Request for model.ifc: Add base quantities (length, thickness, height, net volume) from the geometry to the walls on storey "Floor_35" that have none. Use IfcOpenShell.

First a look at what the model holds.

```python
import ifcopenshell
import ifcopenshell.util.element
import ifcopenshell.util.unit

model = ifcopenshell.open("model.ifc")
print(model.schema)
for unit_type in ("LENGTHUNIT", "AREAUNIT", "VOLUMEUNIT"):
    print(unit_type, ifcopenshell.util.unit.calculate_unit_scale(model, unit_type))
storey = next(s for s in model.by_type("IfcBuildingStorey") if s.Name == "Floor_35")
walls = [e for e in ifcopenshell.util.element.get_decomposition(storey) if e.is_a("IfcWall")]
for e in sorted(walls, key=lambda e: e.id()):
    print(e.id(), e.is_a(), e.Name, list(ifcopenshell.util.element.get_psets(e, qtos_only=True)), sep=" | ")
```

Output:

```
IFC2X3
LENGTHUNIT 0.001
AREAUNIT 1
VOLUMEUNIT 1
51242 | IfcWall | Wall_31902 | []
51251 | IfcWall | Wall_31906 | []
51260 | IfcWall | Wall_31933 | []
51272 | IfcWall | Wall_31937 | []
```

```python
import ifcopenshell
import ifcopenshell.api.pset
import ifcopenshell.geom
import ifcopenshell.util.element
import ifcopenshell.util.shape
import ifcopenshell.util.unit

model = ifcopenshell.open("model.ifc")
unit_scale = ifcopenshell.util.unit.calculate_unit_scale(model)
volume_scale = ifcopenshell.util.unit.calculate_unit_scale(model, "VOLUMEUNIT")
settings = ifcopenshell.geom.settings()

storey = next(s for s in model.by_type("IfcBuildingStorey") if s.Name == "Floor_35")
walls = [e for e in ifcopenshell.util.element.get_decomposition(storey) if e.is_a("IfcWall")]

for e in sorted(walls, key=lambda e: e.id()):
    if ifcopenshell.util.element.get_psets(e, qtos_only=True, should_inherit=False):
        continue
    # Geometry comes back in metres, in the element's own axes.
    shape = ifcopenshell.geom.create_shape(settings, e)
    values = {
        "Length": ifcopenshell.util.shape.get_x(shape.geometry) / unit_scale,
        "Width": ifcopenshell.util.shape.get_y(shape.geometry) / unit_scale,
        "Height": ifcopenshell.util.shape.get_z(shape.geometry) / unit_scale,
        "NetVolume": ifcopenshell.util.shape.get_volume(shape.geometry) / volume_scale,
    }
    qto = ifcopenshell.api.pset.add_qto(model, product=e, name="BaseQuantities")
    ifcopenshell.api.pset.edit_qto(model, qto=qto, properties=values)
    print(e.id(), {k: round(v, 3) for k, v in values.items()})

model.write("model-out.ifc")
```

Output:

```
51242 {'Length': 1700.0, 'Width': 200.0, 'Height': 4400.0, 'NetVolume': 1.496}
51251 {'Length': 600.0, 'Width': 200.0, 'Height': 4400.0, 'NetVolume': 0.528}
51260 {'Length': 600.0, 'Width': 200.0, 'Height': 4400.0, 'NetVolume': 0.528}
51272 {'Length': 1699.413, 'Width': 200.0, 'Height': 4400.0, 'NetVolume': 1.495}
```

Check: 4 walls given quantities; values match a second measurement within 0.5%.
